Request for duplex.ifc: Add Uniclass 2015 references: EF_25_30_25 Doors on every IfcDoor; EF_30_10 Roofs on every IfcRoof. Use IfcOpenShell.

First a look at what the model holds.

```python
import ifcopenshell

model = ifcopenshell.open("duplex.ifc")
print(model.schema)
print("classifications:", [c.Name for c in model.by_type("IfcClassification")])
for ifc_class in ("IfcDoor", "IfcRoof", "IfcStair", "IfcWall", "IfcWindow"):
    print(ifc_class, len(model.by_type(ifc_class)))
```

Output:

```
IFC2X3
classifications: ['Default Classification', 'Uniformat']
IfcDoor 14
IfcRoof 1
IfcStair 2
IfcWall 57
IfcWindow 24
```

```python
import ifcopenshell
import ifcopenshell.api.classification

model = ifcopenshell.open("duplex.ifc")

# IFC2X3 requires Source and Edition and has no link from the project to the system.
system = model.create_entity("IfcClassification", Source="NBS", Edition="2015", Name="Uniclass 2015")

codes = {
    "IfcDoor": ("EF_25_30_25", "Doors"),
    "IfcRoof": ("EF_30_10", "Roofs"),
}
for ifc_class, (code, name) in codes.items():
    products = model.by_type(ifc_class)
    ifcopenshell.api.classification.add_reference(
        model, products=products, classification=system, identification=code, name=name
    )
    print(code, len(products))

model.write("duplex_edited.ifc")
```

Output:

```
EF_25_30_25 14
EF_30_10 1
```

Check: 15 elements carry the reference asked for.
